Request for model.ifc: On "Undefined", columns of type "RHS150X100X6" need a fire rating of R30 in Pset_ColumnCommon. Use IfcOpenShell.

First a look at what the model holds.

```python
import ifcopenshell
import ifcopenshell.util.element

model = ifcopenshell.open("model.ifc")
print(model.schema)
storey = next(s for s in model.by_type("IfcBuildingStorey") if s.Name == "Undefined")
columns = [e for e in ifcopenshell.util.element.get_decomposition(storey) if e.is_a("IfcColumn")]
seen = {}
for e in columns:
    element_type = ifcopenshell.util.element.get_type(e)
    key = (element_type.Name if element_type != e and element_type else None, ifcopenshell.util.element.get_pset(e, "Pset_ColumnCommon", "FireRating"))
    seen[key] = seen.get(key, 0) + 1
for (name, value), count in sorted(seen.items(), key=str):
    print(count, "x", name, "|", value)
```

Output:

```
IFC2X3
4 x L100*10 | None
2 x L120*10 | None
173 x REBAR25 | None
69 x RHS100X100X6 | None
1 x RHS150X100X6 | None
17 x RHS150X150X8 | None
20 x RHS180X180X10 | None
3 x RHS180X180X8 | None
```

```python
import ifcopenshell
import ifcopenshell.api.pset
import ifcopenshell.util.element

model = ifcopenshell.open("model.ifc")

storey = next(s for s in model.by_type("IfcBuildingStorey") if s.Name == "Undefined")
columns = [e for e in ifcopenshell.util.element.get_decomposition(storey) if e.is_a("IfcColumn")]

count = 0
for e in columns:
    element_type = ifcopenshell.util.element.get_type(e)
    if element_type in (None, e) or element_type.Name != "RHS150X100X6":
        continue
    # add_pset returns the element's existing set when there is one.
    pset = ifcopenshell.api.pset.add_pset(model, product=e, name="Pset_ColumnCommon")
    ifcopenshell.api.pset.edit_pset(model, pset=pset, properties={"FireRating": "R30"})
    count += 1

print(count, "columns updated")

model.write("model_v2.ifc")
```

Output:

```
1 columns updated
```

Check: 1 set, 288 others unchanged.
